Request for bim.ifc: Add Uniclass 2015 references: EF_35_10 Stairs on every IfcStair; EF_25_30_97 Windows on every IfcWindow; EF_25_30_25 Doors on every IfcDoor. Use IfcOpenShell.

First a look at what the model holds.

```python
import ifcopenshell

model = ifcopenshell.open("bim.ifc")
print(model.schema)
print("classifications:", [c.Name for c in model.by_type("IfcClassification")])
for ifc_class in ("IfcDoor", "IfcRoof", "IfcStair", "IfcWall", "IfcWindow"):
    print(ifc_class, len(model.by_type(ifc_class)))
```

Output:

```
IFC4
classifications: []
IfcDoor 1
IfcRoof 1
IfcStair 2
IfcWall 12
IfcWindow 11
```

```python
import ifcopenshell
import ifcopenshell.api.classification

model = ifcopenshell.open("bim.ifc")

system = ifcopenshell.api.classification.add_classification(model, classification="Uniclass 2015")

codes = {
    "IfcStair": ("EF_35_10", "Stairs"),
    "IfcWindow": ("EF_25_30_97", "Windows"),
    "IfcDoor": ("EF_25_30_25", "Doors"),
}
for ifc_class, (code, name) in codes.items():
    products = model.by_type(ifc_class)
    ifcopenshell.api.classification.add_reference(
        model, products=products, classification=system, identification=code, name=name
    )
    print(code, len(products))

model.write("bim_rev.ifc")
```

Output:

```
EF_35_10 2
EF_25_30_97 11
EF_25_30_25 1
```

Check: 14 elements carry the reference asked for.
